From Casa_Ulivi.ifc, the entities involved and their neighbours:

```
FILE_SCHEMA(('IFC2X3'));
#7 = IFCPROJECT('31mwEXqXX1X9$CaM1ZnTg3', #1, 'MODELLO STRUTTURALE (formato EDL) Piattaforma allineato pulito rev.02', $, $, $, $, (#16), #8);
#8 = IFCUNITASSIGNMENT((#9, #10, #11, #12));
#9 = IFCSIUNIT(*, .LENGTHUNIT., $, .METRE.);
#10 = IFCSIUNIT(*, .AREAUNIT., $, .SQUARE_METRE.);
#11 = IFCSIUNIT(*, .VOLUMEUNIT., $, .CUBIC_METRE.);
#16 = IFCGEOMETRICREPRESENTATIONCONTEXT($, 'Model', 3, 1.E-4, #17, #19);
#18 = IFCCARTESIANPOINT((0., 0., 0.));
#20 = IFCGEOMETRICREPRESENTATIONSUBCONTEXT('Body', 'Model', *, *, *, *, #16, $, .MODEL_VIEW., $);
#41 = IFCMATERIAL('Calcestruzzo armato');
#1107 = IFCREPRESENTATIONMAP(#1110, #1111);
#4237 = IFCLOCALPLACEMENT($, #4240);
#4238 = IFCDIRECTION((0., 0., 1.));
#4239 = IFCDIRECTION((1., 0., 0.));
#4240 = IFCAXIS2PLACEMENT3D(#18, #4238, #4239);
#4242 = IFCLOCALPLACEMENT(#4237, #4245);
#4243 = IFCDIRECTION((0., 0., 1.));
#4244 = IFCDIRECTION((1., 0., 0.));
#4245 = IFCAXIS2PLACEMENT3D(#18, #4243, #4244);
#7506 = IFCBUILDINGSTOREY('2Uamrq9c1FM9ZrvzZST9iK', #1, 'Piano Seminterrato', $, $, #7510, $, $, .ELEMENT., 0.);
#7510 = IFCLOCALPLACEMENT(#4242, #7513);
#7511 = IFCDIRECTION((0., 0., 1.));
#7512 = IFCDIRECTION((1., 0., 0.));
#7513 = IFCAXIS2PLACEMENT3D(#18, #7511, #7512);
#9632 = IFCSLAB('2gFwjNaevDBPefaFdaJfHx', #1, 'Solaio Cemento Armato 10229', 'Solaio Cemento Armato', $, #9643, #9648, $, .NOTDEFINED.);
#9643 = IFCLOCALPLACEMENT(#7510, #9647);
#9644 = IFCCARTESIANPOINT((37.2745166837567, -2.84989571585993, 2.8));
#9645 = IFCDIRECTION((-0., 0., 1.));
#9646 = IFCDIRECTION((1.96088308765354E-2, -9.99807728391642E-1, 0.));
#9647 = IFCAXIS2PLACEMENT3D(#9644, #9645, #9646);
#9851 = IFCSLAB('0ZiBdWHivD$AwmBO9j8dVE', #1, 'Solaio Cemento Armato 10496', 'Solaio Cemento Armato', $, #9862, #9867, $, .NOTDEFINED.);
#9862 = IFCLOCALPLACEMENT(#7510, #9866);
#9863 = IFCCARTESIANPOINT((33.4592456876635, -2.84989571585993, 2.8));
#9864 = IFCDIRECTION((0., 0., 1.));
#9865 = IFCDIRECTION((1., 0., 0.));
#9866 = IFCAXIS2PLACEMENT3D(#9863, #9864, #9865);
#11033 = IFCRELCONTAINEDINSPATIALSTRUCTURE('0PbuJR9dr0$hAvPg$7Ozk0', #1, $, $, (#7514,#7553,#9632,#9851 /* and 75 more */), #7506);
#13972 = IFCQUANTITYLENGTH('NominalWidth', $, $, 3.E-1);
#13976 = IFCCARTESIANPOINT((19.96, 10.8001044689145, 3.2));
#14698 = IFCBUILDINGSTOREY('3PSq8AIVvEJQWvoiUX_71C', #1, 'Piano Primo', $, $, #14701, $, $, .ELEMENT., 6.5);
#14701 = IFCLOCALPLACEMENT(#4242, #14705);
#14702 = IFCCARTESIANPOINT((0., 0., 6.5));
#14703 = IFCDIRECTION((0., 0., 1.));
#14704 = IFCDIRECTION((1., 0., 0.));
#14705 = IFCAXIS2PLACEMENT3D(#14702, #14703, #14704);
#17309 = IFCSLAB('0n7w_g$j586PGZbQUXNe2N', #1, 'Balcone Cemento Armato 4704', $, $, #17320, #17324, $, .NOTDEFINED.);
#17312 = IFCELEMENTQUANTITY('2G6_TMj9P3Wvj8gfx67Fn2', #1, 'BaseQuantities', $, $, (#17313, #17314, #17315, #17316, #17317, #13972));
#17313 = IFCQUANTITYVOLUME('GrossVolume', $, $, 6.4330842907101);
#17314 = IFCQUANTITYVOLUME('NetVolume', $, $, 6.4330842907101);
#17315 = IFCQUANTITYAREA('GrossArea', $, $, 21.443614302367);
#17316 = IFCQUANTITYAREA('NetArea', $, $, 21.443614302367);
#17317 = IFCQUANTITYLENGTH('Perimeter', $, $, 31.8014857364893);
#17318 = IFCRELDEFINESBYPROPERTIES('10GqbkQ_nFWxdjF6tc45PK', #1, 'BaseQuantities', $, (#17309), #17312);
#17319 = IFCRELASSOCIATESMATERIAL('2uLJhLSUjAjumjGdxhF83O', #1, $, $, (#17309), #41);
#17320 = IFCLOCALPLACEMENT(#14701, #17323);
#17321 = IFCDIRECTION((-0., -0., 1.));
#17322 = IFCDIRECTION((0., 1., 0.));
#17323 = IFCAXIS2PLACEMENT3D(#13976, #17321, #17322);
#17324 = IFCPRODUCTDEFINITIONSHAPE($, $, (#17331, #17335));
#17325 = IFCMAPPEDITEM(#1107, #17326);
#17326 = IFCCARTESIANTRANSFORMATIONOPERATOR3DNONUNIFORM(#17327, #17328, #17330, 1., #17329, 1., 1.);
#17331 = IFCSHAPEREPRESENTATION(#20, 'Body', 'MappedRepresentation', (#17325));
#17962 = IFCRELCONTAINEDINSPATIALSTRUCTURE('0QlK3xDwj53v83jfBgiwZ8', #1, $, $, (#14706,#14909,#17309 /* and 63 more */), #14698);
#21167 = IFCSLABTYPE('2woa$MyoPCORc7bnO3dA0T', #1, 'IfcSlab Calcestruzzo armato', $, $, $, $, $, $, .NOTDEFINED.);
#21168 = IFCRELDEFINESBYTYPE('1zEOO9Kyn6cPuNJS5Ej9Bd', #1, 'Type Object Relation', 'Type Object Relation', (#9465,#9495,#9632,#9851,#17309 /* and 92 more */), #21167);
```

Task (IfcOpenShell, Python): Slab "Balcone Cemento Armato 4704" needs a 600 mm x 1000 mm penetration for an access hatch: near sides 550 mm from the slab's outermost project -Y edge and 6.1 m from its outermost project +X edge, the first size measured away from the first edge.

```python
import numpy as np
import ifcopenshell
import ifcopenshell.api.feature
import ifcopenshell.api.geometry
import ifcopenshell.api.pset
import ifcopenshell.api.root
import ifcopenshell.geom
import ifcopenshell.util.element
import ifcopenshell.util.placement
import ifcopenshell.util.representation
import ifcopenshell.util.shape
import ifcopenshell.util.unit

model = ifcopenshell.open("Casa_Ulivi.ifc")
unit_scale = ifcopenshell.util.unit.calculate_unit_scale(model)
area_scale = ifcopenshell.util.unit.calculate_unit_scale(model, "AREAUNIT")
volume_scale = ifcopenshell.util.unit.calculate_unit_scale(model, "VOLUMEUNIT")
settings = ifcopenshell.geom.settings()


def volume(element):
    """Net volume in cubic metres, openings subtracted."""
    shape = ifcopenshell.geom.create_shape(settings, element)
    return ifcopenshell.util.shape.get_volume(shape.geometry)


slab = model.by_guid("0n7w_g$j586PGZbQUXNe2N")
before = volume(slab)

# Extent in the slab's own axes, in metres. The edges named are its -X and -Y sides.
slab_shape = ifcopenshell.geom.create_shape(settings, slab)
vertices = ifcopenshell.util.shape.get_vertices(slab_shape.geometry)
x_min, y_min, bottom = vertices.min(axis=0)
top = vertices[:, 2].max()

opening = ifcopenshell.api.root.create_entity(model, ifc_class="IfcOpeningElement", name="Access hatch opening")
context = ifcopenshell.util.representation.get_context(model, "Model", "Body", "MODEL_VIEW")
width, depth = 0.6, 1
outline = [(0.0, 0.0), (width, 0.0), (width, depth), (0.0, depth), (0.0, 0.0)]
# Overshoot both faces by 50 mm so the cut is clean.
shape = ifcopenshell.api.geometry.add_slab_representation(
    model, context=context, depth=top - bottom + 0.1, polyline=outline
)
ifcopenshell.api.geometry.assign_representation(model, product=opening, representation=shape)

matrix = ifcopenshell.util.placement.get_local_placement(slab.ObjectPlacement)
matrix[:, 3] = matrix @ np.append(np.array([x_min + 0.55, y_min + 6.1, bottom - 0.05]) / unit_scale, 1.0)
ifcopenshell.api.geometry.edit_object_placement(model, product=opening, matrix=matrix, is_si=False)
ifcopenshell.api.feature.add_feature(model, feature=opening, element=slab)

after = volume(slab)

# Update the slab's stored quantities.
qto = model.by_id(ifcopenshell.util.element.get_pset(slab, "BaseQuantities", should_inherit=False)["id"])
ifcopenshell.api.pset.edit_qto(model, qto=qto, properties={
    "NetVolume": after / volume_scale,
    "NetArea": after / (top - bottom) / area_scale,
})

print(f"slab volume {before:.3f} -> {after:.3f} m3")

model.write("Casa_Ulivi_v2.ifc")
```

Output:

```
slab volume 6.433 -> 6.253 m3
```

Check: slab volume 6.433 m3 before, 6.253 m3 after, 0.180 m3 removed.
